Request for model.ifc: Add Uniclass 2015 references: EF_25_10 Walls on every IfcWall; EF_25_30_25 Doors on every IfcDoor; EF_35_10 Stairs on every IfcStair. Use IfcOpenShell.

First a look at what the model holds.

```python
import ifcopenshell

model = ifcopenshell.open("model.ifc")
print(model.schema)
print("classifications:", [c.Name for c in model.by_type("IfcClassification")])
for ifc_class in ("IfcDoor", "IfcRoof", "IfcStair", "IfcWall", "IfcWindow"):
    print(ifc_class, len(model.by_type(ifc_class)))
```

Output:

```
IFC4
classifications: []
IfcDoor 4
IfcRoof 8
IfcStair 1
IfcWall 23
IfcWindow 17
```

```python
import ifcopenshell
import ifcopenshell.api.classification

model = ifcopenshell.open("model.ifc")

system = ifcopenshell.api.classification.add_classification(model, classification="Uniclass 2015")

codes = {
    "IfcWall": ("EF_25_10", "Walls"),
    "IfcDoor": ("EF_25_30_25", "Doors"),
    "IfcStair": ("EF_35_10", "Stairs"),
}
for ifc_class, (code, name) in codes.items():
    products = model.by_type(ifc_class)
    ifcopenshell.api.classification.add_reference(
        model, products=products, classification=system, identification=code, name=name
    )
    print(code, len(products))

model.write("model_updated.ifc")
```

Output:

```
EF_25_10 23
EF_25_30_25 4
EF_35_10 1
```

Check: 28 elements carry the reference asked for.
